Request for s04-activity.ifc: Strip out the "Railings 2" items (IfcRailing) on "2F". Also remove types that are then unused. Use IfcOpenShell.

First a look at what the model holds.

```python
import ifcopenshell
import ifcopenshell.util.element

model = ifcopenshell.open("s04-activity.ifc")
print(model.schema)
storey = next(s for s in model.by_type("IfcBuildingStorey") if s.Name == "2F")
railings = [e for e in ifcopenshell.util.element.get_decomposition(storey) if e.is_a("IfcRailing")]
seen = {}
for e in railings:
    element_type = ifcopenshell.util.element.get_type(e)
    name = element_type.Name if element_type not in (None, e) else None
    seen[name] = seen.get(name, 0) + 1
for name, count in sorted(seen.items(), key=str):
    print(count, "x", name)
```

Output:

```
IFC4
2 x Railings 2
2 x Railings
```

```python
import ifcopenshell
import ifcopenshell.api.root
import ifcopenshell.util.element

model = ifcopenshell.open("s04-activity.ifc")

storey = next(s for s in model.by_type("IfcBuildingStorey") if s.Name == "2F")
railings = [e for e in ifcopenshell.util.element.get_decomposition(storey) if e.is_a("IfcRailing")]
targets = [e for e in railings if (t := ifcopenshell.util.element.get_type(e)) not in (None, e) and t.Name == "Railings 2"]
types = {ifcopenshell.util.element.get_type(e) for e in targets} - {None, *targets}

for e in targets:
    ifcopenshell.api.root.remove_product(model, product=e)
print(len(targets), "removed")

unused = [t for t in types if not ifcopenshell.util.element.get_types(t)]
for t in unused:
    ifcopenshell.api.root.remove_product(model, product=t)
print(len(unused), "unused types removed")

model.write("s04-activity_updated.ifc")
```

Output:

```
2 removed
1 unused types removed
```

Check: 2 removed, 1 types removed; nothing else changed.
